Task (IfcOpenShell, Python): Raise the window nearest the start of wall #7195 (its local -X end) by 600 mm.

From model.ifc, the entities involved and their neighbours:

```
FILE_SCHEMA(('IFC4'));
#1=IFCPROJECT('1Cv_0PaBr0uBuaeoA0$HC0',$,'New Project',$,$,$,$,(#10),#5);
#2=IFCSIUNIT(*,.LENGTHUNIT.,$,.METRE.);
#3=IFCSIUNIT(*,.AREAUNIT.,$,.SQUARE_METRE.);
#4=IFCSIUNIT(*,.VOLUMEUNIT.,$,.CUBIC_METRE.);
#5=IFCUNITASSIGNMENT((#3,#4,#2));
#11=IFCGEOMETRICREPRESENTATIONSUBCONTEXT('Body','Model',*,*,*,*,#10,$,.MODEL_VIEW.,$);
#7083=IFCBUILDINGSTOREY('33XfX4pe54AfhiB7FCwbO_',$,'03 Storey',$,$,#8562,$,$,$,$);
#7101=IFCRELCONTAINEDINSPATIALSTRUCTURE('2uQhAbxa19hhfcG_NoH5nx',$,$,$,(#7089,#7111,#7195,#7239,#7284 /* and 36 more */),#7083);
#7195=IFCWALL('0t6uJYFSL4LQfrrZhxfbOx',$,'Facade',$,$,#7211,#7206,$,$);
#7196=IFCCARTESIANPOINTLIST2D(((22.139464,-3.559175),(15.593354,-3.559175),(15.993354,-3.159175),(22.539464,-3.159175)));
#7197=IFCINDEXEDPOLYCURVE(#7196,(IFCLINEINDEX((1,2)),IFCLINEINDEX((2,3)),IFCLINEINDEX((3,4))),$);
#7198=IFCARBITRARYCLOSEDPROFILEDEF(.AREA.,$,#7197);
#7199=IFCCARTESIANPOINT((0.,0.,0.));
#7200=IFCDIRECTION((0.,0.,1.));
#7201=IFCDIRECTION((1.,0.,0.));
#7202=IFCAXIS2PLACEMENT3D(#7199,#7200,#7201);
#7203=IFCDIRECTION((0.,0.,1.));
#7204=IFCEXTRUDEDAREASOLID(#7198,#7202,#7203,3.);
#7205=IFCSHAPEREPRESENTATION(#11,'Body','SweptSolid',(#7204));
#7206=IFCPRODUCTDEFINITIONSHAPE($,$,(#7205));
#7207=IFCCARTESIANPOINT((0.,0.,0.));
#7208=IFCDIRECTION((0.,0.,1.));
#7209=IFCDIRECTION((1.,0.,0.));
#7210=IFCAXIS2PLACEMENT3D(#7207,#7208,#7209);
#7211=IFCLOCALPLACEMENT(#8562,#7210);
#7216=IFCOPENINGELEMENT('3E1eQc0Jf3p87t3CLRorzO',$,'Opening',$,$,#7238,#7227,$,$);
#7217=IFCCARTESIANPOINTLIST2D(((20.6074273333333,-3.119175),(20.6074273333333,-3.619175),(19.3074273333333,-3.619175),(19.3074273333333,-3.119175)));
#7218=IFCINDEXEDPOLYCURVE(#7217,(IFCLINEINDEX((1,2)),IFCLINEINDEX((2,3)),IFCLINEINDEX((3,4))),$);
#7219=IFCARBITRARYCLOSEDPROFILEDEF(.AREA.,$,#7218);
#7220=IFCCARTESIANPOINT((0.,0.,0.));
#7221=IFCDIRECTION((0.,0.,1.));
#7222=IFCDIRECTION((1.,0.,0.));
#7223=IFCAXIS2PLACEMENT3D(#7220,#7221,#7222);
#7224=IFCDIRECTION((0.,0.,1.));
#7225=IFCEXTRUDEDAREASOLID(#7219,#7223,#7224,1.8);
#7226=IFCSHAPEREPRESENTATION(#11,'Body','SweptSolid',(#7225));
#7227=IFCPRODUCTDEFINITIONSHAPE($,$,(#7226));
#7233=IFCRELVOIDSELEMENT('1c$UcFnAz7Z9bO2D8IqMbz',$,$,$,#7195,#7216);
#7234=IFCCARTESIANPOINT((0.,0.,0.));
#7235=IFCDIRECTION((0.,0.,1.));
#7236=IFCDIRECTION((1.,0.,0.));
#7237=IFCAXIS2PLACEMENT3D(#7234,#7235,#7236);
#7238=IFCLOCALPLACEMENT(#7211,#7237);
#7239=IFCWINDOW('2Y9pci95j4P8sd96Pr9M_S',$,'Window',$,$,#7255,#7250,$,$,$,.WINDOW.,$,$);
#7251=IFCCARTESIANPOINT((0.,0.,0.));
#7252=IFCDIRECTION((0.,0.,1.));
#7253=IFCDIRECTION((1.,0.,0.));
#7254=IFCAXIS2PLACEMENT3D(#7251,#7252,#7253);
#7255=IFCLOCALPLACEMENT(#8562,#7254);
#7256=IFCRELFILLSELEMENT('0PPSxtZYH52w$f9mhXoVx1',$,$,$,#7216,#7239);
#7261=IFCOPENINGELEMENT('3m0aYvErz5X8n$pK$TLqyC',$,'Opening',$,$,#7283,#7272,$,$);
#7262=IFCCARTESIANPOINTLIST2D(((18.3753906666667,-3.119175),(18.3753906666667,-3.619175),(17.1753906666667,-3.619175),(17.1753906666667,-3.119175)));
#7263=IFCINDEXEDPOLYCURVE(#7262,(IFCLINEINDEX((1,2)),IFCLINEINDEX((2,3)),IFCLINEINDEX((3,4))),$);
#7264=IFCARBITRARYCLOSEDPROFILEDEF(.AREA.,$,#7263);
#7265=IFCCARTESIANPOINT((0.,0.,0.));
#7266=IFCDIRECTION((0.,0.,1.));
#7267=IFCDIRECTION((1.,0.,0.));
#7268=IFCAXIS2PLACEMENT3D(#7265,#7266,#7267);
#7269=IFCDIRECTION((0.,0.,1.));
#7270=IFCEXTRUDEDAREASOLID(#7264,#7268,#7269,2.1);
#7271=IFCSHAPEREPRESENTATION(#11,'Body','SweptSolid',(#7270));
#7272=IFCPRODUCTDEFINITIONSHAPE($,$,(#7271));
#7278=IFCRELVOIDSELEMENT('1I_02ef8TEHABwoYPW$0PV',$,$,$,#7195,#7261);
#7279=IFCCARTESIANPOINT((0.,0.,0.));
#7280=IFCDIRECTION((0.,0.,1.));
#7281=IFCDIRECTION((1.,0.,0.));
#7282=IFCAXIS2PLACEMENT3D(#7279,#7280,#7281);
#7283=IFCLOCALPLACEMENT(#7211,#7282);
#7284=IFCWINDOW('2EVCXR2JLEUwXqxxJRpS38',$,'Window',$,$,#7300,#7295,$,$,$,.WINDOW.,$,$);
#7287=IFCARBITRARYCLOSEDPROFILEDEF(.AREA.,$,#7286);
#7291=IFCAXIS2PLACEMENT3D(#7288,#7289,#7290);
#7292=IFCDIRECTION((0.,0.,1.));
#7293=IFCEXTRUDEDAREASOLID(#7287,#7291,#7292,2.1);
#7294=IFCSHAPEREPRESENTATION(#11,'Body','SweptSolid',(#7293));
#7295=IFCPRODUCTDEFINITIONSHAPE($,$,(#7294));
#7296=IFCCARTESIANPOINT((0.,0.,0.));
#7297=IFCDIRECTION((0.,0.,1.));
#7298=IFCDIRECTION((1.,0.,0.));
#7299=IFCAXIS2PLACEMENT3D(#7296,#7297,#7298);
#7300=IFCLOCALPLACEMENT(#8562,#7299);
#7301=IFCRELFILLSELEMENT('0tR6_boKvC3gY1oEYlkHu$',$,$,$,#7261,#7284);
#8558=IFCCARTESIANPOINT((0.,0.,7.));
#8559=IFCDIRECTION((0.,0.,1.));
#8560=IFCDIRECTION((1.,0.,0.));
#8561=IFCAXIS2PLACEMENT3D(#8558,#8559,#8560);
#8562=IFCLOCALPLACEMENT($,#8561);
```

```python
import numpy as np
import ifcopenshell
import ifcopenshell.api.geometry
import ifcopenshell.util.placement
import ifcopenshell.util.unit

model = ifcopenshell.open("model.ifc")
unit_scale = ifcopenshell.util.unit.calculate_unit_scale(model)

window = model.by_id(7284)
opening = window.FillsVoids[0].RelatingOpeningElement
dz = 0.6

shift = np.array([0.0, 0.0, dz])
# The window is not placed relative to its opening, so move both.
for product in (opening, window):
    matrix = ifcopenshell.util.placement.get_local_placement(product.ObjectPlacement)
    matrix[:3, 3] += shift
    ifcopenshell.api.geometry.edit_object_placement(model, product=product, matrix=matrix, is_si=False)

print(f"moved by {dz * unit_scale:+.3f} m")

model.write("model_rev.ifc")
```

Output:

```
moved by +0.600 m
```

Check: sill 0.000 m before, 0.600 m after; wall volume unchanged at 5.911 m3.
